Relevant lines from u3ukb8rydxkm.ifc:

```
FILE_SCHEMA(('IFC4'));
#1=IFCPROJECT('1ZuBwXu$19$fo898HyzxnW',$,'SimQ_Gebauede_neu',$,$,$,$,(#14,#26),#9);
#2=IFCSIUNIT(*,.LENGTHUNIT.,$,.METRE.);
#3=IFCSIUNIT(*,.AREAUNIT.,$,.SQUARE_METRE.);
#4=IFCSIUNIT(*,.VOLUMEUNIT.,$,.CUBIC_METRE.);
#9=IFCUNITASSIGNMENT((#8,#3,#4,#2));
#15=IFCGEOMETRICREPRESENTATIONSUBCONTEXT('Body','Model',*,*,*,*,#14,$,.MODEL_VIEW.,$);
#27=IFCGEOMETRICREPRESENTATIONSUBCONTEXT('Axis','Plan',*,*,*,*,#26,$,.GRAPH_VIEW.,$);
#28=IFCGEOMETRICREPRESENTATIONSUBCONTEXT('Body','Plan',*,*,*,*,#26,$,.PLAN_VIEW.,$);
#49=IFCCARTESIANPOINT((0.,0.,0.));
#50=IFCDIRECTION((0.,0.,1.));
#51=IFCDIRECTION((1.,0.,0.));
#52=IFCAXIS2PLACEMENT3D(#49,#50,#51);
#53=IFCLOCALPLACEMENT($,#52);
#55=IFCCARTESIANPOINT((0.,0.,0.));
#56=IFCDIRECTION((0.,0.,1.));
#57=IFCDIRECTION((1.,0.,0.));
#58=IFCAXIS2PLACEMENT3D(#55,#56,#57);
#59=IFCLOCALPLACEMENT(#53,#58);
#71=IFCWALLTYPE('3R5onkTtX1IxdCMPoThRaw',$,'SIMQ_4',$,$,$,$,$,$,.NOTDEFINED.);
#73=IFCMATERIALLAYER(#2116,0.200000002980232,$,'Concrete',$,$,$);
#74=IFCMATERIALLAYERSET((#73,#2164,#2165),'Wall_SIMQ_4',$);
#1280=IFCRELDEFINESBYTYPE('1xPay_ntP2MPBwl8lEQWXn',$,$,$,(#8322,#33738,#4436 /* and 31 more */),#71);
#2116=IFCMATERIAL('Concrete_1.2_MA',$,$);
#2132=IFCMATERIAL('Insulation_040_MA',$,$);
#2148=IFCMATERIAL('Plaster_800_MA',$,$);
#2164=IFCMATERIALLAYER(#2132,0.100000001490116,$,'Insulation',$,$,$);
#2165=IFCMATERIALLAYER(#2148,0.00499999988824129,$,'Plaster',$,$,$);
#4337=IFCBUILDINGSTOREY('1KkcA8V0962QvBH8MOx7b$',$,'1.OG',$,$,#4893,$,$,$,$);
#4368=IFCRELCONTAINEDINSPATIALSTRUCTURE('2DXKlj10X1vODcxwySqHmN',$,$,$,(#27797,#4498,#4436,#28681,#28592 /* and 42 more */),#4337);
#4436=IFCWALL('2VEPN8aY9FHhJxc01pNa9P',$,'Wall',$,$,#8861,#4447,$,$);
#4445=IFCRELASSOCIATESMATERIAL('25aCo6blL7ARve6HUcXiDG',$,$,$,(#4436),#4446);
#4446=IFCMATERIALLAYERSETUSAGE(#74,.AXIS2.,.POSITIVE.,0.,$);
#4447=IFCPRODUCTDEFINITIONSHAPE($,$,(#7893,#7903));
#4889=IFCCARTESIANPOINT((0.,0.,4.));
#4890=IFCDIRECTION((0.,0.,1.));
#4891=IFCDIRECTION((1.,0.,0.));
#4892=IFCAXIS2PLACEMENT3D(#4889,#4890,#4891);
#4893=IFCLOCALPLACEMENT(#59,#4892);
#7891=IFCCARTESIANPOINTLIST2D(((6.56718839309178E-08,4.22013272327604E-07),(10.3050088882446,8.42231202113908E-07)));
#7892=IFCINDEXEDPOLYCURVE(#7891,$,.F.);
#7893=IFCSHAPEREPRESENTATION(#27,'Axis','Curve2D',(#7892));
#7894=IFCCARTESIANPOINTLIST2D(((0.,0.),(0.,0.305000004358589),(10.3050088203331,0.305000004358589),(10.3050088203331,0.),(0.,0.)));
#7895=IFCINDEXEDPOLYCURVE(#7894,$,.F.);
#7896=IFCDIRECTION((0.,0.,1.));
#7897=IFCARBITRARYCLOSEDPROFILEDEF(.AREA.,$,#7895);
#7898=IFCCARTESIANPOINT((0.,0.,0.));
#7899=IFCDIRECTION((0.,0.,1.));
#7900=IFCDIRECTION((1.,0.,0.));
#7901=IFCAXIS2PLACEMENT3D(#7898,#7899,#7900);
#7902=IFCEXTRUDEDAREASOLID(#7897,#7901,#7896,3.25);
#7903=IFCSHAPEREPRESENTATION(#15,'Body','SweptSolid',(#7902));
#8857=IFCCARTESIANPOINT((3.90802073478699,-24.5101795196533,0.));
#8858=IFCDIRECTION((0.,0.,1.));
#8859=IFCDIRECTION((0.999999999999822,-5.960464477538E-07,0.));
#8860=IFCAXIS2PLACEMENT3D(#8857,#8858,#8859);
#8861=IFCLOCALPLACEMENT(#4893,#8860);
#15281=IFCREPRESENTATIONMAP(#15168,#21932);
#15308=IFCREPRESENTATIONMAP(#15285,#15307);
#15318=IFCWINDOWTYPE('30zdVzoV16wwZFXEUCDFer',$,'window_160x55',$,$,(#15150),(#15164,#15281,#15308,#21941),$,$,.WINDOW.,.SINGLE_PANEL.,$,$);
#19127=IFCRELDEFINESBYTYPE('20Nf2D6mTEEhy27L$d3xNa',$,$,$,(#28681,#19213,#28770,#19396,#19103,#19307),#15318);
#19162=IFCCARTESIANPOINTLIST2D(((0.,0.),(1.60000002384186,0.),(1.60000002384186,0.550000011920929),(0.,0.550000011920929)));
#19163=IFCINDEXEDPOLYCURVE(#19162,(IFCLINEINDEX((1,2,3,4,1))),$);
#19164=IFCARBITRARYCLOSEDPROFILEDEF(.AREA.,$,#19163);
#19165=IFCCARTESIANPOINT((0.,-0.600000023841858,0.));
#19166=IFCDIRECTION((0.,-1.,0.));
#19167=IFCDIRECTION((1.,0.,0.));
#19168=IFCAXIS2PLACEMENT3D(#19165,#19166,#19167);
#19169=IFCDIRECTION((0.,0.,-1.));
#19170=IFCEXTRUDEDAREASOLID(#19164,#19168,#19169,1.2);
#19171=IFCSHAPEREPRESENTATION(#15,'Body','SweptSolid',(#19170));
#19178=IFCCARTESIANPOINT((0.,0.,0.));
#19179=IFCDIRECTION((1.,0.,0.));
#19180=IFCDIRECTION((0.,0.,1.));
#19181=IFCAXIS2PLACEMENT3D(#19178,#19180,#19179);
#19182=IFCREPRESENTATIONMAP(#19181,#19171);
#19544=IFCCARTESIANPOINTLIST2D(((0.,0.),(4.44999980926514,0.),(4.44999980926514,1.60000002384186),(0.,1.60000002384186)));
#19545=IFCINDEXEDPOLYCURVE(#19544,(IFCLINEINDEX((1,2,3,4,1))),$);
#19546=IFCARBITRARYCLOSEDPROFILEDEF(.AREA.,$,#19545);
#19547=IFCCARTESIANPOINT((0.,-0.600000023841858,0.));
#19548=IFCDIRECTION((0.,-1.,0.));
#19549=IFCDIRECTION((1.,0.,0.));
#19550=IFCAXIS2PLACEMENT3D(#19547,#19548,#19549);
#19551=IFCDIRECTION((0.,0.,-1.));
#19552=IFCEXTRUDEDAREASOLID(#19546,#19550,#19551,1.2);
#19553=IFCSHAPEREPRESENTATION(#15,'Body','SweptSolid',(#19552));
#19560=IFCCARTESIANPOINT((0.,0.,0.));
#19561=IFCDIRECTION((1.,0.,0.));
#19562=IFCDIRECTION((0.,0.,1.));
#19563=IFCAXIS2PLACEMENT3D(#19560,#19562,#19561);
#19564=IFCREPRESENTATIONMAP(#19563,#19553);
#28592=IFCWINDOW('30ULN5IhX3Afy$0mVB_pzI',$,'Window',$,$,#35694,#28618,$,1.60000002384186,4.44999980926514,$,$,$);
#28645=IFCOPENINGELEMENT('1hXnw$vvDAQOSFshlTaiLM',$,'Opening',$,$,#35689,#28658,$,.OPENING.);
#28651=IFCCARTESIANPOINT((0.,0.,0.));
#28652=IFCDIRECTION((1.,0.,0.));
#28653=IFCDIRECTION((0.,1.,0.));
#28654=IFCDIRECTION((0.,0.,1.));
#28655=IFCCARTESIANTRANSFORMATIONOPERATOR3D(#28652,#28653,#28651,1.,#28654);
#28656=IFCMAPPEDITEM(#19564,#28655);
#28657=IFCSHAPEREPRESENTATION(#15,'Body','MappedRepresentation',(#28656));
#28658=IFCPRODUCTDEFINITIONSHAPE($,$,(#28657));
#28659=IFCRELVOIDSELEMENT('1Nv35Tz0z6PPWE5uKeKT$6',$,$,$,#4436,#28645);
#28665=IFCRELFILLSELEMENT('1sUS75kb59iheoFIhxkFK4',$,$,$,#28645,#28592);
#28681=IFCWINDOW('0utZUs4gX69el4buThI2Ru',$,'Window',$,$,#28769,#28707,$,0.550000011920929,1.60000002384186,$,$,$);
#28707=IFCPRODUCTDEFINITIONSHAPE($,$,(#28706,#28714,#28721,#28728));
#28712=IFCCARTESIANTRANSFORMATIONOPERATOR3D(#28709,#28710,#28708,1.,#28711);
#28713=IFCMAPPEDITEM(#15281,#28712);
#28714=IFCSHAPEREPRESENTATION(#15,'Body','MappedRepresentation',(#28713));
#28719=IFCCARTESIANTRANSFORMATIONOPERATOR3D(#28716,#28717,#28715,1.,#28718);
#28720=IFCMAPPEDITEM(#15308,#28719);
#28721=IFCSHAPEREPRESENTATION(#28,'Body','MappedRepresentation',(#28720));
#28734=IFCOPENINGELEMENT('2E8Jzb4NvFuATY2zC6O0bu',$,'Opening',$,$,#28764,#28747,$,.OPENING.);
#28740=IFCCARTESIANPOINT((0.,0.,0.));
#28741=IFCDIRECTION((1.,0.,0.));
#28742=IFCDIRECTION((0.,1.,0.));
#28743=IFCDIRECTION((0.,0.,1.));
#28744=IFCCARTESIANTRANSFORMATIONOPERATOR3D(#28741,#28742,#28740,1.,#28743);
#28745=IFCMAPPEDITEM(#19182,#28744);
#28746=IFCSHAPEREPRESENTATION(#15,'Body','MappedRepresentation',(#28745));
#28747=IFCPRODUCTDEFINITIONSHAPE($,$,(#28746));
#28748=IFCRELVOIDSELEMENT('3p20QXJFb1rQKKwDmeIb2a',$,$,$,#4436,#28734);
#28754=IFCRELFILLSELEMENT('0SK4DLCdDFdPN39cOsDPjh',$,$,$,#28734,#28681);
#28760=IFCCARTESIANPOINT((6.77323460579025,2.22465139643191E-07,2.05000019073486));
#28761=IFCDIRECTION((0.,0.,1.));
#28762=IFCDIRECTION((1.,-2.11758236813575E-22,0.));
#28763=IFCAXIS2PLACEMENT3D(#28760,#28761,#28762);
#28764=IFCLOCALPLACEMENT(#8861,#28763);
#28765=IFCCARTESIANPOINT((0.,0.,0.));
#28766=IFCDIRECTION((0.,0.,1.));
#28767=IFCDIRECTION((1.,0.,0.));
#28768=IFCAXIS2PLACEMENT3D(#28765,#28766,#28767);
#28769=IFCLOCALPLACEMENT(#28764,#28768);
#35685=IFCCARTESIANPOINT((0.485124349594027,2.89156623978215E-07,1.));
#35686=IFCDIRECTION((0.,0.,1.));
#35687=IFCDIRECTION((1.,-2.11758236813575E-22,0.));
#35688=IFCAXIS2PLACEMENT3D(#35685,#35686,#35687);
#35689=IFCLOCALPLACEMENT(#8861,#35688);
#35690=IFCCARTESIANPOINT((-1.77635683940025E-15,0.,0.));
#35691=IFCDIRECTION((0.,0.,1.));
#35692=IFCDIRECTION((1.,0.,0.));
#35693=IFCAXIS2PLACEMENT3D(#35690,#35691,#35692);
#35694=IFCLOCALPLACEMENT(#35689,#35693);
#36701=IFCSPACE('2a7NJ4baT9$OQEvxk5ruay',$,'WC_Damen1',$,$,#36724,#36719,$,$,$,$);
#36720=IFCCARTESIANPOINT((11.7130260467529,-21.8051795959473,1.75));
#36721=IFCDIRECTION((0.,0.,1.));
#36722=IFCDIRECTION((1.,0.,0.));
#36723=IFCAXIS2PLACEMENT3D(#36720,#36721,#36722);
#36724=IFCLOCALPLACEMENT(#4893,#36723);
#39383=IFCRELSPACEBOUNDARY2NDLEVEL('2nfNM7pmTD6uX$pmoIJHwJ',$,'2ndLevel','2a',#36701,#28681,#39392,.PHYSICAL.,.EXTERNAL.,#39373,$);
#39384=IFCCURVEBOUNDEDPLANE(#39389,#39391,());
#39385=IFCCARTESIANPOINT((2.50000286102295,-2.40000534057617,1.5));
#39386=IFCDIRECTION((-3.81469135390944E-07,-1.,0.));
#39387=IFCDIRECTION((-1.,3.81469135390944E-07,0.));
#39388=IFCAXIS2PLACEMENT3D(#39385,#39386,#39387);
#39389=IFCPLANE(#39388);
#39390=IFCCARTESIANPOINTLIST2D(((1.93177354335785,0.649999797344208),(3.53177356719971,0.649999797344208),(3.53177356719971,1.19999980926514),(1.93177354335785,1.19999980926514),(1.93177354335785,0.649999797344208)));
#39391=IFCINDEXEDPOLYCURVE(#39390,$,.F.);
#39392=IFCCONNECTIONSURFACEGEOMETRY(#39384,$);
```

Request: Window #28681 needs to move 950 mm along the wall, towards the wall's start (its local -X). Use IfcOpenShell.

```python
import numpy as np
import ifcopenshell
import ifcopenshell.api.geometry
import ifcopenshell.util.placement
import ifcopenshell.util.unit

model = ifcopenshell.open("u3ukb8rydxkm.ifc")
unit_scale = ifcopenshell.util.unit.calculate_unit_scale(model)

window = model.by_id(28681)
opening = window.FillsVoids[0].RelatingOpeningElement
wall = opening.VoidsElements[0].RelatingBuildingElement

wall_matrix = ifcopenshell.util.placement.get_local_placement(wall.ObjectPlacement)
shift = wall_matrix[:3, 0] * -0.95 / unit_scale
before = ifcopenshell.util.placement.get_local_placement(window.ObjectPlacement)[:3, 3].copy()

# The window is placed relative to its opening, so it follows when the opening moves.
matrix = ifcopenshell.util.placement.get_local_placement(opening.ObjectPlacement)
matrix[:3, 3] += shift
ifcopenshell.api.geometry.edit_object_placement(
    model, product=opening, matrix=matrix, is_si=False, should_transform_children=True
)

# Space boundary surfaces are stored in each space's coordinates; move them too.
for rel in window.ProvidesBoundaries:
    if not rel.ConnectionGeometry:
        continue
    surface = rel.ConnectionGeometry.SurfaceOnRelatingElement.BasisSurface
    space_matrix = ifcopenshell.util.placement.get_local_placement(rel.RelatingSpace.ObjectPlacement)
    point = np.array(surface.Position.Location.Coordinates) + space_matrix[:3, :3].T @ shift
    surface.Position = model.createIfcAxis2Placement3D(
        model.createIfcCartesianPoint(point.tolist()), surface.Position.Axis, surface.Position.RefDirection
    )

after = ifcopenshell.util.placement.get_local_placement(window.ObjectPlacement)[:3, 3]
print("window moved by", (after - before).round(3) + 0.0)

model.write("u3ukb8rydxkm_v2.ifc")
```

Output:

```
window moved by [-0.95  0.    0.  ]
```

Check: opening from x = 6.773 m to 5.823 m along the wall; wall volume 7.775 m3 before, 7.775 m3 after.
